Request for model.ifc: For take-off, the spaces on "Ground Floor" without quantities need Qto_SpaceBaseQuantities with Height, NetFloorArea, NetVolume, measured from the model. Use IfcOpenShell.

First a look at what the model holds.

```python
import ifcopenshell
import ifcopenshell.util.element
import ifcopenshell.util.unit

model = ifcopenshell.open("model.ifc")
print(model.schema)
for unit_type in ("LENGTHUNIT", "AREAUNIT", "VOLUMEUNIT"):
    print(unit_type, ifcopenshell.util.unit.calculate_unit_scale(model, unit_type))
storey = next(s for s in model.by_type("IfcBuildingStorey") if s.Name == "Ground Floor")
spaces = [e for e in ifcopenshell.util.element.get_decomposition(storey) if e.is_a("IfcSpace")]
for e in sorted(spaces, key=lambda e: e.id()):
    print(e.id(), e.is_a(), e.Name, list(ifcopenshell.util.element.get_psets(e, qtos_only=True)), sep=" | ")
```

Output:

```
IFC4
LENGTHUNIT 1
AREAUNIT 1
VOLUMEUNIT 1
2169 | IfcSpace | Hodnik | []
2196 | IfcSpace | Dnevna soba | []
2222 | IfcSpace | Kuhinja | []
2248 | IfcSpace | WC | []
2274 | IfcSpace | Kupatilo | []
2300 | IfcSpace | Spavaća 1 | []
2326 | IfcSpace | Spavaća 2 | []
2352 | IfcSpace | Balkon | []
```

```python
import ifcopenshell
import ifcopenshell.api.pset
import ifcopenshell.geom
import ifcopenshell.util.element
import ifcopenshell.util.shape
import ifcopenshell.util.unit

model = ifcopenshell.open("model.ifc")
unit_scale = ifcopenshell.util.unit.calculate_unit_scale(model)
area_scale = ifcopenshell.util.unit.calculate_unit_scale(model, "AREAUNIT")
volume_scale = ifcopenshell.util.unit.calculate_unit_scale(model, "VOLUMEUNIT")
settings = ifcopenshell.geom.settings()

storey = next(s for s in model.by_type("IfcBuildingStorey") if s.Name == "Ground Floor")
spaces = [e for e in ifcopenshell.util.element.get_decomposition(storey) if e.is_a("IfcSpace")]

for e in sorted(spaces, key=lambda e: e.id()):
    if ifcopenshell.util.element.get_psets(e, qtos_only=True, should_inherit=False):
        continue
    # Geometry comes back in metres, in the element's own axes.
    shape = ifcopenshell.geom.create_shape(settings, e)
    values = {
        "Height": ifcopenshell.util.shape.get_z(shape.geometry) / unit_scale,
        "NetFloorArea": ifcopenshell.util.shape.get_footprint_area(shape.geometry) / area_scale,
        "NetVolume": ifcopenshell.util.shape.get_volume(shape.geometry) / volume_scale,
    }
    qto = ifcopenshell.api.pset.add_qto(model, product=e, name="Qto_SpaceBaseQuantities")
    ifcopenshell.api.pset.edit_qto(model, qto=qto, properties=values)
    print(e.id(), {k: round(v, 3) for k, v in values.items()})

model.write("model_rev.ifc")
```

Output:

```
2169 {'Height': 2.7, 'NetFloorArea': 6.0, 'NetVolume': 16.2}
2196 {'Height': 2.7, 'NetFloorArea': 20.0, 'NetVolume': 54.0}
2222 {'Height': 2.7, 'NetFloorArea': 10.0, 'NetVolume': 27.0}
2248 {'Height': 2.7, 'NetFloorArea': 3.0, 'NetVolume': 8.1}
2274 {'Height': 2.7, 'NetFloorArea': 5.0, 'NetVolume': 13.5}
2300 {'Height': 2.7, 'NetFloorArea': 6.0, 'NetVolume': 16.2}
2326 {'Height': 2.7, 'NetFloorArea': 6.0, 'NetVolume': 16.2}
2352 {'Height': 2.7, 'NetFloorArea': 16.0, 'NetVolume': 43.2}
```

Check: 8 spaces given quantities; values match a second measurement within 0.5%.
